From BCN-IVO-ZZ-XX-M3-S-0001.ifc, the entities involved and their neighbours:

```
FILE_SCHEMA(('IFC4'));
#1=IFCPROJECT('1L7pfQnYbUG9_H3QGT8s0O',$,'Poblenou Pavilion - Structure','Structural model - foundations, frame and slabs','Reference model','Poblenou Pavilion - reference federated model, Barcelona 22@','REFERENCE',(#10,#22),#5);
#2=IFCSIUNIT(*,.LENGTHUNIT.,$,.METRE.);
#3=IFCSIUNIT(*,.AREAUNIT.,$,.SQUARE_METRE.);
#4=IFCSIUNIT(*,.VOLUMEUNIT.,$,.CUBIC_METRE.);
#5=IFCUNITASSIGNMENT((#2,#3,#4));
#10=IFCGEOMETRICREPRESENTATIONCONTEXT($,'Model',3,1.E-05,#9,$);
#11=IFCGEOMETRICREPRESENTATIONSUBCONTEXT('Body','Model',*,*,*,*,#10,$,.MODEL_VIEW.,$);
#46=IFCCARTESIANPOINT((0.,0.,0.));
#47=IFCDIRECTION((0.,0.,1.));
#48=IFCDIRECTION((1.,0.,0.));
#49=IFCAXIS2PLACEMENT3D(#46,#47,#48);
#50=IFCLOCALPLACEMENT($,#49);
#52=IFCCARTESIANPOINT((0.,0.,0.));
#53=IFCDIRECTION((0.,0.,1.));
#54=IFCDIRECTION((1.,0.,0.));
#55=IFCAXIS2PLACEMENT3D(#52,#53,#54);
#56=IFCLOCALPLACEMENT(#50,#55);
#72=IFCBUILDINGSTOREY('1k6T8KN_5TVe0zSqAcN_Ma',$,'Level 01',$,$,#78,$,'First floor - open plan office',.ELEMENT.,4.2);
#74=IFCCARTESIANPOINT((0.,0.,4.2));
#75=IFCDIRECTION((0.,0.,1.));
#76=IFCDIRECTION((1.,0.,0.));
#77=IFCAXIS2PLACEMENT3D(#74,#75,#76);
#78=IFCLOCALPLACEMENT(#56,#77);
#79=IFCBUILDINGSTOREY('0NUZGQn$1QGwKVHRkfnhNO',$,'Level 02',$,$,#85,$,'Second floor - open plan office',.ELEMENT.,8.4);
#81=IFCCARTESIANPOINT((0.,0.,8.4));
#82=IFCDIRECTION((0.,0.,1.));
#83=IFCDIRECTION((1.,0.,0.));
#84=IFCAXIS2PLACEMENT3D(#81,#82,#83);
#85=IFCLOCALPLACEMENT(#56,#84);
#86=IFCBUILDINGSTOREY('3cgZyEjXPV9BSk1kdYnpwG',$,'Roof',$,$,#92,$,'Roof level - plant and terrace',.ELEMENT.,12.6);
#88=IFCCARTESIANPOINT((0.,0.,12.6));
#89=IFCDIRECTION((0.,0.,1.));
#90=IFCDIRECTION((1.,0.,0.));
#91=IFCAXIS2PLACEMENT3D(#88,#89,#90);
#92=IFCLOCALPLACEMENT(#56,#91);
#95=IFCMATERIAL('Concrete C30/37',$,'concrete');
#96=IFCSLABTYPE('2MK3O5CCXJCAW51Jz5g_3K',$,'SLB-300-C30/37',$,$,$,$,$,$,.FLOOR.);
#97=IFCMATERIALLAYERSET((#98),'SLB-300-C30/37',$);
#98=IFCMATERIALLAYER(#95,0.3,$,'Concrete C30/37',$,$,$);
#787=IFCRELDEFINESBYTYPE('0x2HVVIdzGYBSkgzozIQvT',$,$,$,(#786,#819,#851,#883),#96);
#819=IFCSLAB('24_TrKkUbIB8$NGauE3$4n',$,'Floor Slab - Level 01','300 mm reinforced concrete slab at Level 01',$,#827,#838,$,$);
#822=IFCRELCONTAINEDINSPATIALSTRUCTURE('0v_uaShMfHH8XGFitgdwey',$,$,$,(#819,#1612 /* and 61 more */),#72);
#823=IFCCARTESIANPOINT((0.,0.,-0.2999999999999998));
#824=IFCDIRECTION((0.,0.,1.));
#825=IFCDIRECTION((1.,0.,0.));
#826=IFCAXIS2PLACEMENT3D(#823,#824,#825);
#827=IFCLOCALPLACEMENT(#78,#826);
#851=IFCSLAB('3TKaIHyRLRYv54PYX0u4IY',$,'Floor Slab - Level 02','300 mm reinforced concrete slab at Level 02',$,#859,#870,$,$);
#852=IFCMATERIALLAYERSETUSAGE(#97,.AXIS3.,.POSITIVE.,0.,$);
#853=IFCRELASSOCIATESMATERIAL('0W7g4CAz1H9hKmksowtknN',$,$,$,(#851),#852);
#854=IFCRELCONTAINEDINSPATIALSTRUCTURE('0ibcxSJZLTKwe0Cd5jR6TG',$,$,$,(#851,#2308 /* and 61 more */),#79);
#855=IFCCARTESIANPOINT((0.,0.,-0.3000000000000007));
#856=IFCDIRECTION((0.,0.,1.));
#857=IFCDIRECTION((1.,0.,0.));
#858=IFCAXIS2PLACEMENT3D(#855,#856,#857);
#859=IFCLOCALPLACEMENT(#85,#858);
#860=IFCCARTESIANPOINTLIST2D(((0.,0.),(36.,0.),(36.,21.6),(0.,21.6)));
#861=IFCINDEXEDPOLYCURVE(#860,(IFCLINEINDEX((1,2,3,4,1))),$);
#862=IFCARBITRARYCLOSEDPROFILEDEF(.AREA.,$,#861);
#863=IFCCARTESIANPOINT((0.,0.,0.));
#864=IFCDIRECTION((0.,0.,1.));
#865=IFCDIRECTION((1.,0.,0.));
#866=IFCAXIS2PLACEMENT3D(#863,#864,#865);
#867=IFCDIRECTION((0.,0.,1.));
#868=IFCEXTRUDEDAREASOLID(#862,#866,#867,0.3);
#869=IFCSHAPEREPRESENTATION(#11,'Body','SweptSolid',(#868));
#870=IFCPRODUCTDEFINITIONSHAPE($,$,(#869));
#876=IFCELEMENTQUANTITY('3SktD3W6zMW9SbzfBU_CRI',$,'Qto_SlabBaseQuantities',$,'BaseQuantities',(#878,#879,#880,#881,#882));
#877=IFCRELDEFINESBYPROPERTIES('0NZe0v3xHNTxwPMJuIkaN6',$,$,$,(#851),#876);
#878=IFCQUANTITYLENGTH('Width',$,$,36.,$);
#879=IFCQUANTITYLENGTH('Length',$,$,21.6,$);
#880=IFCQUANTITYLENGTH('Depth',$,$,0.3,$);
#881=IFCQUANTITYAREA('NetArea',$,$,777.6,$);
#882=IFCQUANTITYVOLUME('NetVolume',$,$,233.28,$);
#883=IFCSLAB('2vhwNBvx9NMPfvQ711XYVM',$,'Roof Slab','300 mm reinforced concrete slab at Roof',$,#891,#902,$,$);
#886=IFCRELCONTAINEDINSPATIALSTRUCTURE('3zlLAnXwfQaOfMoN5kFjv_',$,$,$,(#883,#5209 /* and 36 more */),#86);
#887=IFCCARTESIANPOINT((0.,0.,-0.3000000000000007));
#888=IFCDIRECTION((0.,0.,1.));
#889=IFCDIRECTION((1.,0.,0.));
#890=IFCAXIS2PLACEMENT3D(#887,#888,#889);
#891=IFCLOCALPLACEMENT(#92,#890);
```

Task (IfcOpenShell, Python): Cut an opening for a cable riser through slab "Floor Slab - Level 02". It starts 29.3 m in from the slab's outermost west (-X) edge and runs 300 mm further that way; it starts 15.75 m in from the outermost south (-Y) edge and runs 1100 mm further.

```python
import numpy as np
import ifcopenshell
import ifcopenshell.api.feature
import ifcopenshell.api.geometry
import ifcopenshell.api.pset
import ifcopenshell.api.root
import ifcopenshell.geom
import ifcopenshell.util.element
import ifcopenshell.util.placement
import ifcopenshell.util.representation
import ifcopenshell.util.shape
import ifcopenshell.util.unit

model = ifcopenshell.open("BCN-IVO-ZZ-XX-M3-S-0001.ifc")
unit_scale = ifcopenshell.util.unit.calculate_unit_scale(model)
area_scale = ifcopenshell.util.unit.calculate_unit_scale(model, "AREAUNIT")
volume_scale = ifcopenshell.util.unit.calculate_unit_scale(model, "VOLUMEUNIT")
settings = ifcopenshell.geom.settings()


def volume(element):
    """Net volume in cubic metres, openings subtracted."""
    shape = ifcopenshell.geom.create_shape(settings, element)
    return ifcopenshell.util.shape.get_volume(shape.geometry)


slab = model.by_guid("3TKaIHyRLRYv54PYX0u4IY")
before = volume(slab)

# Extent in the slab's own axes, in metres. The edges named are its -X and -Y sides.
slab_shape = ifcopenshell.geom.create_shape(settings, slab)
vertices = ifcopenshell.util.shape.get_vertices(slab_shape.geometry)
x_min, y_min, bottom = vertices.min(axis=0)
top = vertices[:, 2].max()

opening = ifcopenshell.api.root.create_entity(model, ifc_class="IfcOpeningElement", name="Cable riser opening", predefined_type="OPENING")
context = ifcopenshell.util.representation.get_context(model, "Model", "Body", "MODEL_VIEW")
width, depth = 0.3, 1.1
outline = [(0.0, 0.0), (width, 0.0), (width, depth), (0.0, depth), (0.0, 0.0)]
# Overshoot both faces by 50 mm so the cut is clean.
shape = ifcopenshell.api.geometry.add_slab_representation(
    model, context=context, depth=top - bottom + 0.1, polyline=outline
)
ifcopenshell.api.geometry.assign_representation(model, product=opening, representation=shape)

matrix = ifcopenshell.util.placement.get_local_placement(slab.ObjectPlacement)
matrix[:, 3] = matrix @ np.append(np.array([x_min + 29.3, y_min + 15.75, bottom - 0.05]) / unit_scale, 1.0)
ifcopenshell.api.geometry.edit_object_placement(model, product=opening, matrix=matrix, is_si=False)
ifcopenshell.api.feature.add_feature(model, feature=opening, element=slab)

after = volume(slab)

# Update the slab's stored quantities.
qto = model.by_id(ifcopenshell.util.element.get_pset(slab, "Qto_SlabBaseQuantities", should_inherit=False)["id"])
ifcopenshell.api.pset.edit_qto(model, qto=qto, properties={
    "NetArea": after / (top - bottom) / area_scale,
    "NetVolume": after / volume_scale,
})

print(f"slab volume {before:.3f} -> {after:.3f} m3")

model.write("BCN-IVO-ZZ-XX-M3-S-0001_updated.ifc")
```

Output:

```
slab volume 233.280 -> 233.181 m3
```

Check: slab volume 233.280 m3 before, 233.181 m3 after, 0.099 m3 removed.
